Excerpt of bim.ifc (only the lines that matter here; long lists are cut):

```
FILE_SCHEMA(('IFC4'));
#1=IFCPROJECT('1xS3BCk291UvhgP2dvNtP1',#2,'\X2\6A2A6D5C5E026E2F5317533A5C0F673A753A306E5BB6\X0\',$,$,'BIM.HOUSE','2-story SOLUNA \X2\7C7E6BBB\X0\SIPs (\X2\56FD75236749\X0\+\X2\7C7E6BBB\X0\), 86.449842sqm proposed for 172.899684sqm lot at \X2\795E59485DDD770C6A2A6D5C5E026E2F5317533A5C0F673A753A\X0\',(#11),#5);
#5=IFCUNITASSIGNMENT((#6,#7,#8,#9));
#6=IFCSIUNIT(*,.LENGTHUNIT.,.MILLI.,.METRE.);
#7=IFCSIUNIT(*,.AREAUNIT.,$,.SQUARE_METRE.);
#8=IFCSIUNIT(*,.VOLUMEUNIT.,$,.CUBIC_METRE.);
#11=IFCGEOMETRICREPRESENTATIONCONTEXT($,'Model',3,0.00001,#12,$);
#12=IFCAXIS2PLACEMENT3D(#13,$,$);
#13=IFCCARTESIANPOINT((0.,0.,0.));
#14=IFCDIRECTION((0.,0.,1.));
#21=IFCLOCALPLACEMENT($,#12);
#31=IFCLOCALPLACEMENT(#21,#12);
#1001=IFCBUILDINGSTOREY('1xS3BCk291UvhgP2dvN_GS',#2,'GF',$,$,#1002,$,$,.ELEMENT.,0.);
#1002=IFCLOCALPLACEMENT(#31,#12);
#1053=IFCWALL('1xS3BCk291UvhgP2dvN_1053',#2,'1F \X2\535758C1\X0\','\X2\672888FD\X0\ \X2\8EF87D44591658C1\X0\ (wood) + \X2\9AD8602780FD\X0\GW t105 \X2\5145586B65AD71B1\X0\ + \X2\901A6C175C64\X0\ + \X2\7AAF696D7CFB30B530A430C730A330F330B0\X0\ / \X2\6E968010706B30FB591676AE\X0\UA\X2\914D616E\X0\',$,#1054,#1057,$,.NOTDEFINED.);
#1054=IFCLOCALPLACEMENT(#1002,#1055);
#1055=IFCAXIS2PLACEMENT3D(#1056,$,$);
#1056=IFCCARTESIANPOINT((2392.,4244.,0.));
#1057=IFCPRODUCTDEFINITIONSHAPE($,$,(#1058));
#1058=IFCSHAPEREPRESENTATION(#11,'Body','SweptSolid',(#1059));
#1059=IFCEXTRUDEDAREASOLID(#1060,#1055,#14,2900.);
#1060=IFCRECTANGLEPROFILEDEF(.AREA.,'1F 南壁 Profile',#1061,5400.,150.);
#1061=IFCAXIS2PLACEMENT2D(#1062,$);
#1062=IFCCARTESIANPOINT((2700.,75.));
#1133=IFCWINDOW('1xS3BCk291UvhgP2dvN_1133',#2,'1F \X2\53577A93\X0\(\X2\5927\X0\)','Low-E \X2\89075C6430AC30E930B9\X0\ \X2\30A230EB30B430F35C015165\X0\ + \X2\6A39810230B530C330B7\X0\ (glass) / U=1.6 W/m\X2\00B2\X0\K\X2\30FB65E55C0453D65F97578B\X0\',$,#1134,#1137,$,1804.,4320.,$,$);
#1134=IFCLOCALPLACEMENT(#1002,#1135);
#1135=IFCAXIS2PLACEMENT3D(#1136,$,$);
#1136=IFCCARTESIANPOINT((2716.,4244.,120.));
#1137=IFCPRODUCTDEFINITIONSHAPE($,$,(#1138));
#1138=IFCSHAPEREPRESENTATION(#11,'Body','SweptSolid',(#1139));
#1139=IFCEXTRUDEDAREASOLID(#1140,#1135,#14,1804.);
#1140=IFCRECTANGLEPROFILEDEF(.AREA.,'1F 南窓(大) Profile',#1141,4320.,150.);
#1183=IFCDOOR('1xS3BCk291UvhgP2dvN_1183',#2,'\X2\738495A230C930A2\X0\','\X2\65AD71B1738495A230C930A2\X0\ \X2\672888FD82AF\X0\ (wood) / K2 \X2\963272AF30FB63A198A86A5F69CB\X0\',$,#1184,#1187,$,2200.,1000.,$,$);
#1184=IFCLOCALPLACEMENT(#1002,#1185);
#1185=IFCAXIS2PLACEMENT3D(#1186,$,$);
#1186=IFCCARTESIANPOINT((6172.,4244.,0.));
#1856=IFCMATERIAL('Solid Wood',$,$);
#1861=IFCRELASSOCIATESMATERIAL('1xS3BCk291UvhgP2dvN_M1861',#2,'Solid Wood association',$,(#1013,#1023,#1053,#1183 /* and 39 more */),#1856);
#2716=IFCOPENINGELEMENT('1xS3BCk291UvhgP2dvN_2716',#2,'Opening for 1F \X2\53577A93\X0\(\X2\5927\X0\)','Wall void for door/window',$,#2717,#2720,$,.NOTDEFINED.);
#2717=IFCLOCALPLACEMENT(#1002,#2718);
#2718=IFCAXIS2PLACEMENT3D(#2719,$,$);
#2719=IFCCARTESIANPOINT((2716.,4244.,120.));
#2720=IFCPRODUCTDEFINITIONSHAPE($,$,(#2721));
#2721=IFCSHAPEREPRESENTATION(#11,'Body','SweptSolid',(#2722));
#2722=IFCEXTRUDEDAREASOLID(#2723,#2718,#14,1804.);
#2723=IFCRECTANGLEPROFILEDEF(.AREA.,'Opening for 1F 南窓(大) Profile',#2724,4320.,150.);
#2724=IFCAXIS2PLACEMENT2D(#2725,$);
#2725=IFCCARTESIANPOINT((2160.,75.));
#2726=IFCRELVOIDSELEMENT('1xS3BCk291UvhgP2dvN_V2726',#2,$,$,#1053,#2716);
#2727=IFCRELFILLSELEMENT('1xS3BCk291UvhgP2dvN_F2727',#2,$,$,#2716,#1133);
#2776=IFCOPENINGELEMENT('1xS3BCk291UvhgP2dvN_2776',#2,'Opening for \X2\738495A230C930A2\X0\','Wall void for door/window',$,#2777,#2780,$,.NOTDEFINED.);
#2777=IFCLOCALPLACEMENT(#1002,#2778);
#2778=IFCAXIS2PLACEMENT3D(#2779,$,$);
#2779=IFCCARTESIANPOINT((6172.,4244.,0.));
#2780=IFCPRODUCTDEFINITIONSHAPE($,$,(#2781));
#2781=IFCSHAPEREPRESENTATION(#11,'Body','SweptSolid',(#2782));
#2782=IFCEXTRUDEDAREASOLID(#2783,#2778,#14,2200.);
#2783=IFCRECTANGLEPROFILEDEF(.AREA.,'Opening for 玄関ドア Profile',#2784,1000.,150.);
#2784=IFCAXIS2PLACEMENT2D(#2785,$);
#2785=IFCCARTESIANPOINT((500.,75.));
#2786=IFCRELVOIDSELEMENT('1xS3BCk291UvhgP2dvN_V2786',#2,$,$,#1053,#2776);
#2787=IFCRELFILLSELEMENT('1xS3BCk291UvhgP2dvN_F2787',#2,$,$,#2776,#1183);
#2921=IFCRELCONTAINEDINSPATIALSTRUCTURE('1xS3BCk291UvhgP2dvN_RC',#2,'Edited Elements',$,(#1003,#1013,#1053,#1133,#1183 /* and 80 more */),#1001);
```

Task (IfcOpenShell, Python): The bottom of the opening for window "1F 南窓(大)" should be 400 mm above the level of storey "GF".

```python
import numpy as np
import ifcopenshell
import ifcopenshell.api.geometry
import ifcopenshell.geom
import ifcopenshell.util.element
import ifcopenshell.util.placement
import ifcopenshell.util.shape
import ifcopenshell.util.unit

model = ifcopenshell.open("bim.ifc")
unit_scale = ifcopenshell.util.unit.calculate_unit_scale(model)

window = model.by_id(1133)
opening = window.FillsVoids[0].RelatingOpeningElement
storey = ifcopenshell.util.element.get_container(window, ifc_class="IfcBuildingStorey")
level = ifcopenshell.util.placement.get_local_placement(storey.ObjectPlacement)[2, 3]

# The opening's origin need not be at the sill, so measure its lowest point.
shape = ifcopenshell.geom.create_shape(ifcopenshell.geom.settings(), opening)
bottom = ifcopenshell.util.shape.get_shape_bottom_elevation(shape, shape.geometry) / unit_scale
dz = level + 400.0 - bottom

shift = np.array([0.0, 0.0, dz])
# The window is not placed relative to its opening, so move both.
for product in (opening, window):
    matrix = ifcopenshell.util.placement.get_local_placement(product.ObjectPlacement)
    matrix[:3, 3] += shift
    ifcopenshell.api.geometry.edit_object_placement(model, product=product, matrix=matrix, is_si=False)

print(f"moved by {dz * unit_scale:+.3f} m")

model.write("bim_v2.ifc")
```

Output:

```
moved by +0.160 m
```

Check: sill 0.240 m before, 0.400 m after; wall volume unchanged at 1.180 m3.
